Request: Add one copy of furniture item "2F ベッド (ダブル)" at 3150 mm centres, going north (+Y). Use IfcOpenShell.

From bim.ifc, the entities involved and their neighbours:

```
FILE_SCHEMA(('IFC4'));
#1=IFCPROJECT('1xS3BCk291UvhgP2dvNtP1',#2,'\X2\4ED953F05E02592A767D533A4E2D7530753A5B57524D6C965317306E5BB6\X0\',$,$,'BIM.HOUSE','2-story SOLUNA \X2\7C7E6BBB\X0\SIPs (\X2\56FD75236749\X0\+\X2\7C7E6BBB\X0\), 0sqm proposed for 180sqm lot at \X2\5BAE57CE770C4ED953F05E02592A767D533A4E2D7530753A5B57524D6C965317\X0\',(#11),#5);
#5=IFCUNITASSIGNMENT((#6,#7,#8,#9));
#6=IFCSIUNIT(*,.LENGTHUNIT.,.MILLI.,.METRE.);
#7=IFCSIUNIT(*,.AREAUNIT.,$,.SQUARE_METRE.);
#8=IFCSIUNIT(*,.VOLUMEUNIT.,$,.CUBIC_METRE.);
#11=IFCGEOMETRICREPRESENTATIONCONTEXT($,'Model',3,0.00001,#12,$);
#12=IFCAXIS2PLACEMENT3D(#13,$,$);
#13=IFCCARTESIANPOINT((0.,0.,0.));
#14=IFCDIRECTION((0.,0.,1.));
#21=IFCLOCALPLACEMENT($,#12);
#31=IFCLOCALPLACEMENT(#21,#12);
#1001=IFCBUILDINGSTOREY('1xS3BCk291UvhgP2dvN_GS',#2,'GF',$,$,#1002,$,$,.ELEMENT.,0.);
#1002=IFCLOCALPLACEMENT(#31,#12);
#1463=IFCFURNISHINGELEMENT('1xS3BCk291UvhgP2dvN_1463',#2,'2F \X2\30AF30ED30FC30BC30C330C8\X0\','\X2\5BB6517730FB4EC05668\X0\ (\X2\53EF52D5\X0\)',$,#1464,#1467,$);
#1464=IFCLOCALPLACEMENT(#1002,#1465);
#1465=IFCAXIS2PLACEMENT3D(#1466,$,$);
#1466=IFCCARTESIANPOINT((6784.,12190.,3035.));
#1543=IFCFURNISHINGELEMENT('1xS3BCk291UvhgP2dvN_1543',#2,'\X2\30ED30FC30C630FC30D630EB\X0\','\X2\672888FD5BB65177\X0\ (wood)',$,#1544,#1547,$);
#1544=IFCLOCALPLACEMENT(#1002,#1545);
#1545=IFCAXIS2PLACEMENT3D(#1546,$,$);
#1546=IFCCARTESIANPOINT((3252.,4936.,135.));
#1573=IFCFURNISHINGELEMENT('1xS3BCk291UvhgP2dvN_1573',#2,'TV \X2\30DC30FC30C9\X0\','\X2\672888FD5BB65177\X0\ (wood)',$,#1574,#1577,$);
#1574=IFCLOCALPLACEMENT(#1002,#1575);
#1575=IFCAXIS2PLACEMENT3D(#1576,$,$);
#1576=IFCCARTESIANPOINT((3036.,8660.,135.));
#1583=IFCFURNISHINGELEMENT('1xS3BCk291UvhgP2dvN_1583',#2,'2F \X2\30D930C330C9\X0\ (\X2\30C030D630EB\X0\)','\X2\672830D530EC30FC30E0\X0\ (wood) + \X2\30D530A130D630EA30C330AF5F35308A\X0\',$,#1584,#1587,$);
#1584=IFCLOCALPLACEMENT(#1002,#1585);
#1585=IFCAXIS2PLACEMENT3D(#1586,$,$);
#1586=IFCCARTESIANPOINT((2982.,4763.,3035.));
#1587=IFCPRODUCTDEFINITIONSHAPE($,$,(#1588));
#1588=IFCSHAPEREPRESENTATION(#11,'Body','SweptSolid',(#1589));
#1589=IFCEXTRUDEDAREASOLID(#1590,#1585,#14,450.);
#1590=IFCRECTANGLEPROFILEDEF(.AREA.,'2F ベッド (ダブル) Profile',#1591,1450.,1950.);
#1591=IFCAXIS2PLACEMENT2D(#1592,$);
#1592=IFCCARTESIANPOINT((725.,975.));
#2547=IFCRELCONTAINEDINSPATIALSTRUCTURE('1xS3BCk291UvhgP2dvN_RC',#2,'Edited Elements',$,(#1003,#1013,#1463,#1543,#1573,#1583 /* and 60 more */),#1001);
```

```python
import numpy as np
import ifcopenshell
import ifcopenshell.api.geometry
import ifcopenshell.api.root
import ifcopenshell.util.element
import ifcopenshell.util.placement

model = ifcopenshell.open("bim.ifc")


def reuse_history(source, copy):
    """copy_class also copies each property set's owner history, people and application; keep the originals."""
    for rel in copy.IsDefinedBy:
        if rel.is_a("IfcRelDefinesByProperties") and (history := rel.RelatingPropertyDefinition.OwnerHistory):
            rel.RelatingPropertyDefinition.OwnerHistory = source.OwnerHistory
            ifcopenshell.util.element.remove_deep2(model, history)


source = model.by_guid("1xS3BCk291UvhgP2dvN_1583")
base = ifcopenshell.util.placement.get_local_placement(source.ObjectPlacement)
step = np.array([0.0, 1.0, 0.0]) * 3150.0

for i in range(1, 2):
    copy = ifcopenshell.api.root.copy_class(model, product=source)
    copy.Representation = ifcopenshell.util.element.copy_deep(
        model, source.Representation, exclude=["IfcGeometricRepresentationContext", "IfcRepresentationMap"]
    )
    reuse_history(source, copy)
    matrix = base.copy()
    matrix[:3, 3] += i * step
    print("added at", matrix[:3, 3].round(3) + 0.0)
    ifcopenshell.api.geometry.edit_object_placement(model, product=copy, matrix=matrix, is_si=False)

model.write("bim_v2.ifc")
```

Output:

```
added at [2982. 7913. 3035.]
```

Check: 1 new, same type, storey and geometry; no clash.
